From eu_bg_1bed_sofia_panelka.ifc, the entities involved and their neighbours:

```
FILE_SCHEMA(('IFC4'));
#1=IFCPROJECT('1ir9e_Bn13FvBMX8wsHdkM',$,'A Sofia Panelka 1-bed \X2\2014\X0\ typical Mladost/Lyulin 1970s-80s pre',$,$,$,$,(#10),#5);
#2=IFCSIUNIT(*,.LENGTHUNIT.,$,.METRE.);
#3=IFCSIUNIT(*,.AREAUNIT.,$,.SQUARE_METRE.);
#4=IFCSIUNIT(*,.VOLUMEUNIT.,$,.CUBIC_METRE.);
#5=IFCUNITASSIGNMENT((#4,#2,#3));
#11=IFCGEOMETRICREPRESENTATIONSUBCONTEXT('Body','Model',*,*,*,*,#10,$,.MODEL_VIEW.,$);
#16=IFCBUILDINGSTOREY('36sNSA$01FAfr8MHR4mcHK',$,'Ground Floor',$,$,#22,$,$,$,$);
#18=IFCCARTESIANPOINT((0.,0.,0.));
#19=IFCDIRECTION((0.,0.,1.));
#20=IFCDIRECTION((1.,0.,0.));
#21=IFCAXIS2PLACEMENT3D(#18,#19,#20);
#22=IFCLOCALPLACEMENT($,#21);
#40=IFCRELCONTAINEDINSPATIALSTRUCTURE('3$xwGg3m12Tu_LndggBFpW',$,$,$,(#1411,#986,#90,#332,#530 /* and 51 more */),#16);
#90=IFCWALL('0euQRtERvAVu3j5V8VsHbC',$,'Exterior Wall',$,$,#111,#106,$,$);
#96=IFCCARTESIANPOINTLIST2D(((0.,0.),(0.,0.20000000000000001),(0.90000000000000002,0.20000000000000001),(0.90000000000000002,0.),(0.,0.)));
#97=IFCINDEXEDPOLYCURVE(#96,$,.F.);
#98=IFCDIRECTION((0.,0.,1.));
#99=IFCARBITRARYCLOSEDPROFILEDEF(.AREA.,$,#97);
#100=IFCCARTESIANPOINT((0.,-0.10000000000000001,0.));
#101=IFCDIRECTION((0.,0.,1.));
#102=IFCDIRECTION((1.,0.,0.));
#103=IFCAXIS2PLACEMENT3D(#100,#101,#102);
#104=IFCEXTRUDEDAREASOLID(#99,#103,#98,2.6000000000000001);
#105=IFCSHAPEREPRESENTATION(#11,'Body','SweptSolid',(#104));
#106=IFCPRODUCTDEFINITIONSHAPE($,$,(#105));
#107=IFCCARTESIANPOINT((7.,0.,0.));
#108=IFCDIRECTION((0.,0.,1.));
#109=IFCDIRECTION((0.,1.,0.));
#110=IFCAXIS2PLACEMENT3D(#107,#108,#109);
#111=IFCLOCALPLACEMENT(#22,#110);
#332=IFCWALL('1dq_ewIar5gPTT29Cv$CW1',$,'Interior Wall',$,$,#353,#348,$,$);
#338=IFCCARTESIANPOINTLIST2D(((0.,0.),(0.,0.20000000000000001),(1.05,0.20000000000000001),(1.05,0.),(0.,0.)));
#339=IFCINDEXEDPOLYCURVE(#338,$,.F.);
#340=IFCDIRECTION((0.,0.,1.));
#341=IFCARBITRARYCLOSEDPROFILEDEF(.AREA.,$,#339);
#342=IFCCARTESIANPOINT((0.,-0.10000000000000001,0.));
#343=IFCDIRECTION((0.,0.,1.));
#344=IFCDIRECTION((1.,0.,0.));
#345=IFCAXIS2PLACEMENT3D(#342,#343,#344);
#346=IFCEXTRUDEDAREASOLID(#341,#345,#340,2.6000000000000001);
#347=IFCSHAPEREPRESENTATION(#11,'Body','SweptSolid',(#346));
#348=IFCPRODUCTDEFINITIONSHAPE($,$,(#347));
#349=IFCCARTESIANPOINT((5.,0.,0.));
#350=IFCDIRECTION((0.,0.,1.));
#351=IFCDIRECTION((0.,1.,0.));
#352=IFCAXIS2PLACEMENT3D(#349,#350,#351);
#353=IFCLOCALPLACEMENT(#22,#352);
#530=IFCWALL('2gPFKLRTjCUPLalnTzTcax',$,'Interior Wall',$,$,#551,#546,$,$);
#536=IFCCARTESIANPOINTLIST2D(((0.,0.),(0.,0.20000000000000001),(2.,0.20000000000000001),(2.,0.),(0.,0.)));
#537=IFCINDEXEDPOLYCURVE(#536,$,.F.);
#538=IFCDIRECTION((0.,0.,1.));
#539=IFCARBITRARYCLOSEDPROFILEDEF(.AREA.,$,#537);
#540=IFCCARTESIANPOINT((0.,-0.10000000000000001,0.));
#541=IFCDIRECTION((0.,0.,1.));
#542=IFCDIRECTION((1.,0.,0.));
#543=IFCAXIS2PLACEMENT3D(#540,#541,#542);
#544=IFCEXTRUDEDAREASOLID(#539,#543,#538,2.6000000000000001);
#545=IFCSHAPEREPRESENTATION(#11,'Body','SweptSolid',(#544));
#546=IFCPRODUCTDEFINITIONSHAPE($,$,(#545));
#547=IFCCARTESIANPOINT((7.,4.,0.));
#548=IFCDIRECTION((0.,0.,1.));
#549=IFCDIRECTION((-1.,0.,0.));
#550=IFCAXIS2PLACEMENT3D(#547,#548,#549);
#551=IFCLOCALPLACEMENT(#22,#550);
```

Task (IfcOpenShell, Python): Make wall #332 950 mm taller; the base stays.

```python
import ifcopenshell
import ifcopenshell.geom
import ifcopenshell.util.representation
import ifcopenshell.util.shape
import ifcopenshell.util.unit

model = ifcopenshell.open("eu_bg_1bed_sofia_panelka.ifc")
unit_scale = ifcopenshell.util.unit.calculate_unit_scale(model)
settings = ifcopenshell.geom.settings()


def volume(element):
    """Net volume in cubic metres, openings subtracted."""
    shape = ifcopenshell.geom.create_shape(settings, element)
    return ifcopenshell.util.shape.get_volume(shape.geometry)


wall = model.by_guid("1dq_ewIar5gPTT29Cv$CW1")
before = volume(wall)

body = ifcopenshell.util.representation.get_representation(wall, "Model", "Body")
solid = body.Items[0]
old_height = solid.Depth
solid.Depth += 0.95 / unit_scale
after = volume(wall)

print(f"height {old_height:g} -> {solid.Depth:g}, volume {before:.3f} -> {after:.3f} m3")

model.write("eu_bg_1bed_sofia_panelka_v2.ifc")
```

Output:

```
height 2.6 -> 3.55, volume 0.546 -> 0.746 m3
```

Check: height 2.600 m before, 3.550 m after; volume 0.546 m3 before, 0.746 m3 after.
